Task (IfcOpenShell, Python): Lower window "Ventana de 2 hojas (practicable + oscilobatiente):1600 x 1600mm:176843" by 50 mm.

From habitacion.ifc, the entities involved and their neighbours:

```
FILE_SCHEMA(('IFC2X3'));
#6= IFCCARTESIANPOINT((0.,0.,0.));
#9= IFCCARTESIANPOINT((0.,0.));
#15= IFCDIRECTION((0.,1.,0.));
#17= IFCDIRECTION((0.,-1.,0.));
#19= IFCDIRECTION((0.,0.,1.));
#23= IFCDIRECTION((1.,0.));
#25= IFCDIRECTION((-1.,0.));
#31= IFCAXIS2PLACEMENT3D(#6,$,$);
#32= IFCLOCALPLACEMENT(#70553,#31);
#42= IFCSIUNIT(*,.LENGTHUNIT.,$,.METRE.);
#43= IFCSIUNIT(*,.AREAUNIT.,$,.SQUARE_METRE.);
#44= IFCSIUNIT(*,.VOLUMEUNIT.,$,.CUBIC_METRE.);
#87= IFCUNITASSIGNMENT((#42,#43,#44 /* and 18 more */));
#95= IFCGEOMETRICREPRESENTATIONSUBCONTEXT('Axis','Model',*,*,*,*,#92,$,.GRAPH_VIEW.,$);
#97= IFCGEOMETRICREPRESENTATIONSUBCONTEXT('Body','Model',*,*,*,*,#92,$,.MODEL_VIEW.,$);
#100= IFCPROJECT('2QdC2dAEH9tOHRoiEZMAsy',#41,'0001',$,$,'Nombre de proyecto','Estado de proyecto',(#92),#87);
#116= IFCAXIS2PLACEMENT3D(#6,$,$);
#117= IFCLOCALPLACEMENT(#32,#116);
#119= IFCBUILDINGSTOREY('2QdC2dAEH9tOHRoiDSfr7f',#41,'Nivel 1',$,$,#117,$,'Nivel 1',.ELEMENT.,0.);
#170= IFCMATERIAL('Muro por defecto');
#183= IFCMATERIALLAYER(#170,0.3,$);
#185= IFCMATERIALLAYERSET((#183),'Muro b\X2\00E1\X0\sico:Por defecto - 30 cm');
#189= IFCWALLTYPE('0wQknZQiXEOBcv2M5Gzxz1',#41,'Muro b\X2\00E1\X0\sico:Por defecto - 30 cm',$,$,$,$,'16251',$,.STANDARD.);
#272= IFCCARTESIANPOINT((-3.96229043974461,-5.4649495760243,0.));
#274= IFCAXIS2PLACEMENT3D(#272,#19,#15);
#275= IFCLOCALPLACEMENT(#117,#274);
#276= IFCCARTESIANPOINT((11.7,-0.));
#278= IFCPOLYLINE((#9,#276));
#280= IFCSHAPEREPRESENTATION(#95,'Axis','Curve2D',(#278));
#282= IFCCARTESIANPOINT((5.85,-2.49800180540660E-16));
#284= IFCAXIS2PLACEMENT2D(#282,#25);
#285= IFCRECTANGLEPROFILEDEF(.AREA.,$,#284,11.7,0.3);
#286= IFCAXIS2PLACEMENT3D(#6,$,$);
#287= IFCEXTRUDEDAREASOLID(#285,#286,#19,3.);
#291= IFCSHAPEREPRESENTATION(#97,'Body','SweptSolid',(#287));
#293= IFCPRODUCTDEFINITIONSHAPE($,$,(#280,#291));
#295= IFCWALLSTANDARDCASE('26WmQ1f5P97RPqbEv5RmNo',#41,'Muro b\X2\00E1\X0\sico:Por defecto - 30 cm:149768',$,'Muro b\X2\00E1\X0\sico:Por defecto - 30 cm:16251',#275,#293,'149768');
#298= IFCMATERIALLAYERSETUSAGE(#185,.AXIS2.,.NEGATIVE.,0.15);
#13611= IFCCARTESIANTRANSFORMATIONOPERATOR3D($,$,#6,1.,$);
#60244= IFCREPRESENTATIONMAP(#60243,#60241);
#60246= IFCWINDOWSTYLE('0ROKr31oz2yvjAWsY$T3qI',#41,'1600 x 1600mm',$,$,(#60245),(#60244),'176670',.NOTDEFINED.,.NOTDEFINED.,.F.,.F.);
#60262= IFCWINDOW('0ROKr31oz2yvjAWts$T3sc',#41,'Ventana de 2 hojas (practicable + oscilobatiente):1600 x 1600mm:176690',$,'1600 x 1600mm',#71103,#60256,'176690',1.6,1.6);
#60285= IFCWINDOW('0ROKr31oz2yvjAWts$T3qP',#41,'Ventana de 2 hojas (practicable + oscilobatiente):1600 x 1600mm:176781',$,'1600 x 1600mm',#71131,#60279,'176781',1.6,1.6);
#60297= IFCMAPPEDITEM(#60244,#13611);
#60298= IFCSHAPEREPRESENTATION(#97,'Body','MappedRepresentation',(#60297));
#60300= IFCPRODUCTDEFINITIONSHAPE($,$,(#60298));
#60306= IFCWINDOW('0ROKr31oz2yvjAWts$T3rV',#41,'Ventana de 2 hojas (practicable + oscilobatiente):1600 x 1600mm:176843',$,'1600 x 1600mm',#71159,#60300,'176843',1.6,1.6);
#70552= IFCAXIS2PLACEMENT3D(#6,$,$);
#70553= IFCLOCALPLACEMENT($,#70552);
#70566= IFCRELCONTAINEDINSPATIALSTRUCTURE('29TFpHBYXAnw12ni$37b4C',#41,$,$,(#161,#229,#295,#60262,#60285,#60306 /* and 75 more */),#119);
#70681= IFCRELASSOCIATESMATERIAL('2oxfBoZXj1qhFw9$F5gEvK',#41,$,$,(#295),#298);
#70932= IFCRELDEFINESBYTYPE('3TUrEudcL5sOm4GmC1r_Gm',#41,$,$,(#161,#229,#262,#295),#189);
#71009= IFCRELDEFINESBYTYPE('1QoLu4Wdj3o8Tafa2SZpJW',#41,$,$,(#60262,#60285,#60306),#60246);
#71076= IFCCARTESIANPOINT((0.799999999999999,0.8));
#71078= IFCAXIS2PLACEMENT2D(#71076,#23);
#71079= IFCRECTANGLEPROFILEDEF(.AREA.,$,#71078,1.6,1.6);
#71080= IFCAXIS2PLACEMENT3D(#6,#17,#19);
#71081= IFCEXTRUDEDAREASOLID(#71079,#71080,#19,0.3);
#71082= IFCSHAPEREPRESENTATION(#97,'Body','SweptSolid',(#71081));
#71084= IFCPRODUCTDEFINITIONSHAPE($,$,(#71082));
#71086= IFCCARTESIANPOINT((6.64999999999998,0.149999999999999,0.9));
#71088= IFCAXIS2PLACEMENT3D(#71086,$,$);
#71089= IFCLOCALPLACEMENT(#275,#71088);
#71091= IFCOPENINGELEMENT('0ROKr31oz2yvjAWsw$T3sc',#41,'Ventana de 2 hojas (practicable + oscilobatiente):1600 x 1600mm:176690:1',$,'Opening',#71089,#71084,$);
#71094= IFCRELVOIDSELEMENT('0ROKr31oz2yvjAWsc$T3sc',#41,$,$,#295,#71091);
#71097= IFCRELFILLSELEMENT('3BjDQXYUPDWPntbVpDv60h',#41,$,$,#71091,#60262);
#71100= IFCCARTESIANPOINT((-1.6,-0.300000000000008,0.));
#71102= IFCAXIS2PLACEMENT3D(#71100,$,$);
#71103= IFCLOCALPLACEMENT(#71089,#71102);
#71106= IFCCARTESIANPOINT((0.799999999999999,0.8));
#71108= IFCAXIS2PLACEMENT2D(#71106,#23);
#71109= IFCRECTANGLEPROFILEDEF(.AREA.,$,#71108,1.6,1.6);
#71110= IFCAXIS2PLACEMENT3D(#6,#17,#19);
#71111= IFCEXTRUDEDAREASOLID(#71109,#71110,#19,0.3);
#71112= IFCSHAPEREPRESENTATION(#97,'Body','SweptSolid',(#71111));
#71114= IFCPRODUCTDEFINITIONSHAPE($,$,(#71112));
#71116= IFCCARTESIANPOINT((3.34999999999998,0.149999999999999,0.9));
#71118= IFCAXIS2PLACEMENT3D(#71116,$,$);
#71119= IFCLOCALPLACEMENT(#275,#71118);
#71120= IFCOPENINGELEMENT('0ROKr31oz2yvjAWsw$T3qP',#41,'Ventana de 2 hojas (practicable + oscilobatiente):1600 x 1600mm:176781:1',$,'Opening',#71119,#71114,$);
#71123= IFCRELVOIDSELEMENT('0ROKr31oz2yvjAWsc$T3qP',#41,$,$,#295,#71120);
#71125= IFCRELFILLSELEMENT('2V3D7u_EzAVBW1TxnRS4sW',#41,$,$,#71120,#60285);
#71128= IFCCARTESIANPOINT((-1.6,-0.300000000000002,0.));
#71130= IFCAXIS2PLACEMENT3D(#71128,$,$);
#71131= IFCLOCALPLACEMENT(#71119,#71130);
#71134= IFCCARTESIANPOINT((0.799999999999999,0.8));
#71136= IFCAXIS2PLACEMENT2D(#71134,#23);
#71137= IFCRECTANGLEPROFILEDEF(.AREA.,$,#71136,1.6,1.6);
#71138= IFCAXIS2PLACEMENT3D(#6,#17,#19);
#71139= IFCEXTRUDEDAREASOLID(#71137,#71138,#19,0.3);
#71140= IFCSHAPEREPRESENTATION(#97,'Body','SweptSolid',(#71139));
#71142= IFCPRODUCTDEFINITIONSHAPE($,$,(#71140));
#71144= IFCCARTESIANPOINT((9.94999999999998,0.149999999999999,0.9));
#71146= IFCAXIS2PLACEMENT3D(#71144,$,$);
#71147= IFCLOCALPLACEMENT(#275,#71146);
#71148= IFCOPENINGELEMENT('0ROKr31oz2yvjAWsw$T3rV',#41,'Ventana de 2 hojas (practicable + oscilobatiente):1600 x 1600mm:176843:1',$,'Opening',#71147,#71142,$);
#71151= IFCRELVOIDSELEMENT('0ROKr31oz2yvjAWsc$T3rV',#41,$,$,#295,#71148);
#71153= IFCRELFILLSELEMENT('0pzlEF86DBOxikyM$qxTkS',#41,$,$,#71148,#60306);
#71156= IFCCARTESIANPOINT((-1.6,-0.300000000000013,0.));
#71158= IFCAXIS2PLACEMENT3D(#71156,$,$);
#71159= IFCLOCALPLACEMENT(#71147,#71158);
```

```python
import numpy as np
import ifcopenshell
import ifcopenshell.api.geometry
import ifcopenshell.util.placement
import ifcopenshell.util.unit

model = ifcopenshell.open("habitacion.ifc")
unit_scale = ifcopenshell.util.unit.calculate_unit_scale(model)

window = model.by_guid("0ROKr31oz2yvjAWts$T3rV")
opening = window.FillsVoids[0].RelatingOpeningElement
dz = -0.05 / unit_scale

shift = np.array([0.0, 0.0, dz])
# The window is placed relative to its opening, so it follows when the opening moves.
matrix = ifcopenshell.util.placement.get_local_placement(opening.ObjectPlacement)
matrix[:3, 3] += shift
ifcopenshell.api.geometry.edit_object_placement(
    model, product=opening, matrix=matrix, is_si=False, should_transform_children=True
)

print(f"moved by {dz * unit_scale:+.3f} m")

model.write("habitacion_edited.ifc")
```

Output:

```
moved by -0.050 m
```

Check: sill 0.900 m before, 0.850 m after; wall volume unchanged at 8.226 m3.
